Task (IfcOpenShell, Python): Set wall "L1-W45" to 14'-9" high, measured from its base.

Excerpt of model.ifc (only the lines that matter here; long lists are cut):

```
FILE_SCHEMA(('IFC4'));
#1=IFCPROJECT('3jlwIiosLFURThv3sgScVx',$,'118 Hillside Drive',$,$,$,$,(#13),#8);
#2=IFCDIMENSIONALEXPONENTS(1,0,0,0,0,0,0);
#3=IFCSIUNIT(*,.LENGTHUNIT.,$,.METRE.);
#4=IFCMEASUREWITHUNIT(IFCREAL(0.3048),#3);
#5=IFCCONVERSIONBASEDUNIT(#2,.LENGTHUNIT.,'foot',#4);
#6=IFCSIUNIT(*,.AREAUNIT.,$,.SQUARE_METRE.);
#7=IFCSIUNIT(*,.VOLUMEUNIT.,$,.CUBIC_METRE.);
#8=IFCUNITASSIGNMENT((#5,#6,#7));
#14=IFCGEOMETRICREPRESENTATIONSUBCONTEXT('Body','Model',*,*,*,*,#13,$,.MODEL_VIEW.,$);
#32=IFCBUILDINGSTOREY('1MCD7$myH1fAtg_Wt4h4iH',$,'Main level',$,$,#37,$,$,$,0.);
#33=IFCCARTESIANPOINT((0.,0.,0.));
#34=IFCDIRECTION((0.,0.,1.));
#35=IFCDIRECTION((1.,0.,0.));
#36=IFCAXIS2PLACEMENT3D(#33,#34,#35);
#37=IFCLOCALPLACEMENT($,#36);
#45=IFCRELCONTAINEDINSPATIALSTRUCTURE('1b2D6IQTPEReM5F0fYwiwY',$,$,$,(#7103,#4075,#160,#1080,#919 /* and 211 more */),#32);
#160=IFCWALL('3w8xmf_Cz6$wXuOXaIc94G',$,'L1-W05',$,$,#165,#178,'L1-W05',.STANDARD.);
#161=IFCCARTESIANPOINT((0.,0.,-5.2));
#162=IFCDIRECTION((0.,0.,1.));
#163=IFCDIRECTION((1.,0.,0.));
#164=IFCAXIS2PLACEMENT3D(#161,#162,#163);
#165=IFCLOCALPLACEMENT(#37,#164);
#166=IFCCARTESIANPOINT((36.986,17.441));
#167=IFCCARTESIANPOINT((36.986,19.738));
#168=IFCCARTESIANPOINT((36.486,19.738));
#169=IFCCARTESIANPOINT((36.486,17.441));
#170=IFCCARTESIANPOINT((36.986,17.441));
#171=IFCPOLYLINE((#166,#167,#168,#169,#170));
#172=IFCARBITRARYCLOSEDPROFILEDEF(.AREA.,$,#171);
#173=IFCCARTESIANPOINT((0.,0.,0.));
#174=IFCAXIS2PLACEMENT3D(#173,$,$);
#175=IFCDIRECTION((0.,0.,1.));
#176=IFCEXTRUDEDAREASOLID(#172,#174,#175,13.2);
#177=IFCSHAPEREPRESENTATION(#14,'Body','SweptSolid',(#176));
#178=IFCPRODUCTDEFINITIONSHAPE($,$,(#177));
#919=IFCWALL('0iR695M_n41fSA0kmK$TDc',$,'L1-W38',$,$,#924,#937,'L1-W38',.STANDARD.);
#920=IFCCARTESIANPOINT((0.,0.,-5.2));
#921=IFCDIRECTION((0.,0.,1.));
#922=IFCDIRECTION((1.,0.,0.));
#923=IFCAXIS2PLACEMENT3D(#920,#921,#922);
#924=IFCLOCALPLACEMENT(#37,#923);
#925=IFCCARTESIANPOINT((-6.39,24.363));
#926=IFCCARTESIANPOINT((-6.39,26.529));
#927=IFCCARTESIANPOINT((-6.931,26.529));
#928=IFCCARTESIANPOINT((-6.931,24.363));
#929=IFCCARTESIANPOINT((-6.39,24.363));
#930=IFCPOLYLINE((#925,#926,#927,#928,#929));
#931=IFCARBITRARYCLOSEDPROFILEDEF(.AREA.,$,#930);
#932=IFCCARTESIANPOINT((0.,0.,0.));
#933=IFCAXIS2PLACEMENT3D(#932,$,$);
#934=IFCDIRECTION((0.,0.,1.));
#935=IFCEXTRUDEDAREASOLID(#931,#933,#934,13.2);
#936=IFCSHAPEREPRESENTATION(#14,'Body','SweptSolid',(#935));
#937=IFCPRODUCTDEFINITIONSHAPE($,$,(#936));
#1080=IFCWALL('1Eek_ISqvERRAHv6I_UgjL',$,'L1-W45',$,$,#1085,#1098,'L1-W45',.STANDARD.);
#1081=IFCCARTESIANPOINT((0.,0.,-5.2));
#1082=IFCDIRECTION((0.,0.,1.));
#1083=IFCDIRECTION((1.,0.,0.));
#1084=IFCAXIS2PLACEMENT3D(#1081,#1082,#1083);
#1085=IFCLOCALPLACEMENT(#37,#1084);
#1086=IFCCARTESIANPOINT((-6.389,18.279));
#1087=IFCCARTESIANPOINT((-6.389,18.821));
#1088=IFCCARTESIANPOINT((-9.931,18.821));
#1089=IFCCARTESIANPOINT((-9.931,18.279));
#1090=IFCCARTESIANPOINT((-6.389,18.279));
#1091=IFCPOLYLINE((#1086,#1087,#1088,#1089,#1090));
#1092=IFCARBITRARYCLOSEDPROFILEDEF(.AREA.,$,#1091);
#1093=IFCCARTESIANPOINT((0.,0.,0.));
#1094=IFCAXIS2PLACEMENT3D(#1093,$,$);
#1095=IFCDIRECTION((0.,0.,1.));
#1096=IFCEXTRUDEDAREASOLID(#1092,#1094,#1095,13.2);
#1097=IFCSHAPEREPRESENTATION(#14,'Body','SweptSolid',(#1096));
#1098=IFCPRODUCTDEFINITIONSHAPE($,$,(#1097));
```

```python
import ifcopenshell
import ifcopenshell.geom
import ifcopenshell.util.representation
import ifcopenshell.util.shape
import ifcopenshell.util.unit

model = ifcopenshell.open("model.ifc")
unit_scale = ifcopenshell.util.unit.calculate_unit_scale(model)
settings = ifcopenshell.geom.settings()


def volume(element):
    """Net volume in cubic metres, openings subtracted."""
    shape = ifcopenshell.geom.create_shape(settings, element)
    return ifcopenshell.util.shape.get_volume(shape.geometry)


wall = model.by_guid("1Eek_ISqvERRAHv6I_UgjL")
before = volume(wall)

body = ifcopenshell.util.representation.get_representation(wall, "Model", "Body")
solid = body.Items[0]
old_height = solid.Depth
solid.Depth = 177 * 0.0254 / unit_scale
after = volume(wall)

print(f"height {old_height:g} -> {solid.Depth:g}, volume {before:.3f} -> {after:.3f} m3")

model.write("model_rev.ifc")
```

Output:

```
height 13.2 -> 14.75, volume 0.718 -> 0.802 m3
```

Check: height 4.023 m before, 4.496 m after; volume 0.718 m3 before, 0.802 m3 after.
